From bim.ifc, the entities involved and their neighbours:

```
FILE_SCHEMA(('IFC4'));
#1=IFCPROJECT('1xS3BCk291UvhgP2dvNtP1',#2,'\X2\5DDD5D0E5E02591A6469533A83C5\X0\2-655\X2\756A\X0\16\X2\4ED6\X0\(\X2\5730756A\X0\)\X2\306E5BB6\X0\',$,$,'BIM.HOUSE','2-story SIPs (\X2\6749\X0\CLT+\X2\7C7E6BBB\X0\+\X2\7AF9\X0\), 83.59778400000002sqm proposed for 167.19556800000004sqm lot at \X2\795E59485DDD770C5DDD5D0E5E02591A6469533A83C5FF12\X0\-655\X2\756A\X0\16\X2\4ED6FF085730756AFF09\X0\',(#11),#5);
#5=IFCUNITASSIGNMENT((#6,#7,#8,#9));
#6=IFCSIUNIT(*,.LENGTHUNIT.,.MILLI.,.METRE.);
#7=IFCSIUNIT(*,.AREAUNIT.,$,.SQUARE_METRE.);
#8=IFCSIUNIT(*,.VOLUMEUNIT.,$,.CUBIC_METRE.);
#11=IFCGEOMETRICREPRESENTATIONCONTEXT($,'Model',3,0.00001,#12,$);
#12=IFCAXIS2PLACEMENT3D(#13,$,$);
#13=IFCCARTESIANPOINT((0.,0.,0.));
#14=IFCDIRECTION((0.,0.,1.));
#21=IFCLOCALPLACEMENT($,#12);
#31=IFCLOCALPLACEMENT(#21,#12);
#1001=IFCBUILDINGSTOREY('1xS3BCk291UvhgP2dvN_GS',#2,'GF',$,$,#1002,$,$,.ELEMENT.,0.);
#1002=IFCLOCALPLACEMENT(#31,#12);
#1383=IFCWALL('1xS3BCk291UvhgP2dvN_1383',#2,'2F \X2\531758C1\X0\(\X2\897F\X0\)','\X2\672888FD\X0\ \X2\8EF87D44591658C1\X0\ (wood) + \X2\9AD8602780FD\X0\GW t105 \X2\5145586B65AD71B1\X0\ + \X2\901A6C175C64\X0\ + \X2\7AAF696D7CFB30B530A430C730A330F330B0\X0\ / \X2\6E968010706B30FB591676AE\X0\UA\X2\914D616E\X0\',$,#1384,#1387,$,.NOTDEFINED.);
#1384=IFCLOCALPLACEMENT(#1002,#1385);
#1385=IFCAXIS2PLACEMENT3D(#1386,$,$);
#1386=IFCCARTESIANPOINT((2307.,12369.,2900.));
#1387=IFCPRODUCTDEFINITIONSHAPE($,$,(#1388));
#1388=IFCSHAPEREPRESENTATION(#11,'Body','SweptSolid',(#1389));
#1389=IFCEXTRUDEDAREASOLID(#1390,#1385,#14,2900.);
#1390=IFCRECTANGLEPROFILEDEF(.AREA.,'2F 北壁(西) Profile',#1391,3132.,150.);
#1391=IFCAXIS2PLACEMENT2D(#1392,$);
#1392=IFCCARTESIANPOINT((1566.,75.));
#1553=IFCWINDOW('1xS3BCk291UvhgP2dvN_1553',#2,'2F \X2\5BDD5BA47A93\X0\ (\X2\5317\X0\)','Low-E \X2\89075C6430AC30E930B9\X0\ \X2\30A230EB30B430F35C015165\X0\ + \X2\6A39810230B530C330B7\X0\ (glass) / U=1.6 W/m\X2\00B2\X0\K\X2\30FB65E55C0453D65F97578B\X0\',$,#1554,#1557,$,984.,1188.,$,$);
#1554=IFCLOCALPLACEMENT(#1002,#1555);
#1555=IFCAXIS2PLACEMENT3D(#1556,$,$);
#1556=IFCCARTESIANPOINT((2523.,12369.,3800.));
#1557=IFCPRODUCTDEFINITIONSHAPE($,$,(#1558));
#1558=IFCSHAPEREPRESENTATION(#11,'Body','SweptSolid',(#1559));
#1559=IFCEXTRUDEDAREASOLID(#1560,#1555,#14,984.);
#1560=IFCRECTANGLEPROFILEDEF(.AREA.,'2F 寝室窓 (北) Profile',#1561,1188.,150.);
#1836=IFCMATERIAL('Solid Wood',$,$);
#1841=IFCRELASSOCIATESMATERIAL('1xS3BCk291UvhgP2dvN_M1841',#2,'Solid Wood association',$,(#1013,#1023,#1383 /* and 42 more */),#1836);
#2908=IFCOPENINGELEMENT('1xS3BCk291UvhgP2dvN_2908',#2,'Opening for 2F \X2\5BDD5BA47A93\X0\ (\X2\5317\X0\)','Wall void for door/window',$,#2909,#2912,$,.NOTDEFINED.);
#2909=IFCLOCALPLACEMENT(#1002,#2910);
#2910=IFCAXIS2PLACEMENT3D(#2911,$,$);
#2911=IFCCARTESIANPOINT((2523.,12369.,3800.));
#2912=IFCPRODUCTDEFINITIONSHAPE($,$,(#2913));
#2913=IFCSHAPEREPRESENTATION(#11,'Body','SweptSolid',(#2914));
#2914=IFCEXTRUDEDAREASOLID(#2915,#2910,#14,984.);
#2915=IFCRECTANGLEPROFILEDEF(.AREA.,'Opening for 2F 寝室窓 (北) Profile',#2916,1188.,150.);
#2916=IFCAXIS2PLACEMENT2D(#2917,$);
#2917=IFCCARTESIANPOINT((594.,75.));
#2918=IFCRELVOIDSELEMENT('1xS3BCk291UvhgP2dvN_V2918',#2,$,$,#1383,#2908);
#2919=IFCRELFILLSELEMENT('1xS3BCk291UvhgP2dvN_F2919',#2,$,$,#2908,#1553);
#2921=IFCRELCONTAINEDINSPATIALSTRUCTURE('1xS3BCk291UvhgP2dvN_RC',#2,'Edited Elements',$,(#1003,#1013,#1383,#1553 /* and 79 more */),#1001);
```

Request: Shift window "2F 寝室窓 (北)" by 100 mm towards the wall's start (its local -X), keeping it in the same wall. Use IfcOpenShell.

```python
import ifcopenshell
import ifcopenshell.api.geometry
import ifcopenshell.util.placement
import ifcopenshell.util.unit

model = ifcopenshell.open("bim.ifc")
unit_scale = ifcopenshell.util.unit.calculate_unit_scale(model)

window = model.by_id(1553)
opening = window.FillsVoids[0].RelatingOpeningElement
wall = opening.VoidsElements[0].RelatingBuildingElement

wall_matrix = ifcopenshell.util.placement.get_local_placement(wall.ObjectPlacement)
shift = wall_matrix[:3, 0] * -0.1 / unit_scale
before = ifcopenshell.util.placement.get_local_placement(window.ObjectPlacement)[:3, 3].copy()

# The window is not placed relative to its opening, so move both.
for product in (opening, window):
    matrix = ifcopenshell.util.placement.get_local_placement(product.ObjectPlacement)
    matrix[:3, 3] += shift
    ifcopenshell.api.geometry.edit_object_placement(model, product=product, matrix=matrix, is_si=False)

after = ifcopenshell.util.placement.get_local_placement(window.ObjectPlacement)[:3, 3]
print("window moved by", (after - before).round(3) + 0.0)

model.write("bim_updated.ifc")
```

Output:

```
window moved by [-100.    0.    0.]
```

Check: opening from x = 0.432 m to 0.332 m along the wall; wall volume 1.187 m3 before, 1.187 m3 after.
